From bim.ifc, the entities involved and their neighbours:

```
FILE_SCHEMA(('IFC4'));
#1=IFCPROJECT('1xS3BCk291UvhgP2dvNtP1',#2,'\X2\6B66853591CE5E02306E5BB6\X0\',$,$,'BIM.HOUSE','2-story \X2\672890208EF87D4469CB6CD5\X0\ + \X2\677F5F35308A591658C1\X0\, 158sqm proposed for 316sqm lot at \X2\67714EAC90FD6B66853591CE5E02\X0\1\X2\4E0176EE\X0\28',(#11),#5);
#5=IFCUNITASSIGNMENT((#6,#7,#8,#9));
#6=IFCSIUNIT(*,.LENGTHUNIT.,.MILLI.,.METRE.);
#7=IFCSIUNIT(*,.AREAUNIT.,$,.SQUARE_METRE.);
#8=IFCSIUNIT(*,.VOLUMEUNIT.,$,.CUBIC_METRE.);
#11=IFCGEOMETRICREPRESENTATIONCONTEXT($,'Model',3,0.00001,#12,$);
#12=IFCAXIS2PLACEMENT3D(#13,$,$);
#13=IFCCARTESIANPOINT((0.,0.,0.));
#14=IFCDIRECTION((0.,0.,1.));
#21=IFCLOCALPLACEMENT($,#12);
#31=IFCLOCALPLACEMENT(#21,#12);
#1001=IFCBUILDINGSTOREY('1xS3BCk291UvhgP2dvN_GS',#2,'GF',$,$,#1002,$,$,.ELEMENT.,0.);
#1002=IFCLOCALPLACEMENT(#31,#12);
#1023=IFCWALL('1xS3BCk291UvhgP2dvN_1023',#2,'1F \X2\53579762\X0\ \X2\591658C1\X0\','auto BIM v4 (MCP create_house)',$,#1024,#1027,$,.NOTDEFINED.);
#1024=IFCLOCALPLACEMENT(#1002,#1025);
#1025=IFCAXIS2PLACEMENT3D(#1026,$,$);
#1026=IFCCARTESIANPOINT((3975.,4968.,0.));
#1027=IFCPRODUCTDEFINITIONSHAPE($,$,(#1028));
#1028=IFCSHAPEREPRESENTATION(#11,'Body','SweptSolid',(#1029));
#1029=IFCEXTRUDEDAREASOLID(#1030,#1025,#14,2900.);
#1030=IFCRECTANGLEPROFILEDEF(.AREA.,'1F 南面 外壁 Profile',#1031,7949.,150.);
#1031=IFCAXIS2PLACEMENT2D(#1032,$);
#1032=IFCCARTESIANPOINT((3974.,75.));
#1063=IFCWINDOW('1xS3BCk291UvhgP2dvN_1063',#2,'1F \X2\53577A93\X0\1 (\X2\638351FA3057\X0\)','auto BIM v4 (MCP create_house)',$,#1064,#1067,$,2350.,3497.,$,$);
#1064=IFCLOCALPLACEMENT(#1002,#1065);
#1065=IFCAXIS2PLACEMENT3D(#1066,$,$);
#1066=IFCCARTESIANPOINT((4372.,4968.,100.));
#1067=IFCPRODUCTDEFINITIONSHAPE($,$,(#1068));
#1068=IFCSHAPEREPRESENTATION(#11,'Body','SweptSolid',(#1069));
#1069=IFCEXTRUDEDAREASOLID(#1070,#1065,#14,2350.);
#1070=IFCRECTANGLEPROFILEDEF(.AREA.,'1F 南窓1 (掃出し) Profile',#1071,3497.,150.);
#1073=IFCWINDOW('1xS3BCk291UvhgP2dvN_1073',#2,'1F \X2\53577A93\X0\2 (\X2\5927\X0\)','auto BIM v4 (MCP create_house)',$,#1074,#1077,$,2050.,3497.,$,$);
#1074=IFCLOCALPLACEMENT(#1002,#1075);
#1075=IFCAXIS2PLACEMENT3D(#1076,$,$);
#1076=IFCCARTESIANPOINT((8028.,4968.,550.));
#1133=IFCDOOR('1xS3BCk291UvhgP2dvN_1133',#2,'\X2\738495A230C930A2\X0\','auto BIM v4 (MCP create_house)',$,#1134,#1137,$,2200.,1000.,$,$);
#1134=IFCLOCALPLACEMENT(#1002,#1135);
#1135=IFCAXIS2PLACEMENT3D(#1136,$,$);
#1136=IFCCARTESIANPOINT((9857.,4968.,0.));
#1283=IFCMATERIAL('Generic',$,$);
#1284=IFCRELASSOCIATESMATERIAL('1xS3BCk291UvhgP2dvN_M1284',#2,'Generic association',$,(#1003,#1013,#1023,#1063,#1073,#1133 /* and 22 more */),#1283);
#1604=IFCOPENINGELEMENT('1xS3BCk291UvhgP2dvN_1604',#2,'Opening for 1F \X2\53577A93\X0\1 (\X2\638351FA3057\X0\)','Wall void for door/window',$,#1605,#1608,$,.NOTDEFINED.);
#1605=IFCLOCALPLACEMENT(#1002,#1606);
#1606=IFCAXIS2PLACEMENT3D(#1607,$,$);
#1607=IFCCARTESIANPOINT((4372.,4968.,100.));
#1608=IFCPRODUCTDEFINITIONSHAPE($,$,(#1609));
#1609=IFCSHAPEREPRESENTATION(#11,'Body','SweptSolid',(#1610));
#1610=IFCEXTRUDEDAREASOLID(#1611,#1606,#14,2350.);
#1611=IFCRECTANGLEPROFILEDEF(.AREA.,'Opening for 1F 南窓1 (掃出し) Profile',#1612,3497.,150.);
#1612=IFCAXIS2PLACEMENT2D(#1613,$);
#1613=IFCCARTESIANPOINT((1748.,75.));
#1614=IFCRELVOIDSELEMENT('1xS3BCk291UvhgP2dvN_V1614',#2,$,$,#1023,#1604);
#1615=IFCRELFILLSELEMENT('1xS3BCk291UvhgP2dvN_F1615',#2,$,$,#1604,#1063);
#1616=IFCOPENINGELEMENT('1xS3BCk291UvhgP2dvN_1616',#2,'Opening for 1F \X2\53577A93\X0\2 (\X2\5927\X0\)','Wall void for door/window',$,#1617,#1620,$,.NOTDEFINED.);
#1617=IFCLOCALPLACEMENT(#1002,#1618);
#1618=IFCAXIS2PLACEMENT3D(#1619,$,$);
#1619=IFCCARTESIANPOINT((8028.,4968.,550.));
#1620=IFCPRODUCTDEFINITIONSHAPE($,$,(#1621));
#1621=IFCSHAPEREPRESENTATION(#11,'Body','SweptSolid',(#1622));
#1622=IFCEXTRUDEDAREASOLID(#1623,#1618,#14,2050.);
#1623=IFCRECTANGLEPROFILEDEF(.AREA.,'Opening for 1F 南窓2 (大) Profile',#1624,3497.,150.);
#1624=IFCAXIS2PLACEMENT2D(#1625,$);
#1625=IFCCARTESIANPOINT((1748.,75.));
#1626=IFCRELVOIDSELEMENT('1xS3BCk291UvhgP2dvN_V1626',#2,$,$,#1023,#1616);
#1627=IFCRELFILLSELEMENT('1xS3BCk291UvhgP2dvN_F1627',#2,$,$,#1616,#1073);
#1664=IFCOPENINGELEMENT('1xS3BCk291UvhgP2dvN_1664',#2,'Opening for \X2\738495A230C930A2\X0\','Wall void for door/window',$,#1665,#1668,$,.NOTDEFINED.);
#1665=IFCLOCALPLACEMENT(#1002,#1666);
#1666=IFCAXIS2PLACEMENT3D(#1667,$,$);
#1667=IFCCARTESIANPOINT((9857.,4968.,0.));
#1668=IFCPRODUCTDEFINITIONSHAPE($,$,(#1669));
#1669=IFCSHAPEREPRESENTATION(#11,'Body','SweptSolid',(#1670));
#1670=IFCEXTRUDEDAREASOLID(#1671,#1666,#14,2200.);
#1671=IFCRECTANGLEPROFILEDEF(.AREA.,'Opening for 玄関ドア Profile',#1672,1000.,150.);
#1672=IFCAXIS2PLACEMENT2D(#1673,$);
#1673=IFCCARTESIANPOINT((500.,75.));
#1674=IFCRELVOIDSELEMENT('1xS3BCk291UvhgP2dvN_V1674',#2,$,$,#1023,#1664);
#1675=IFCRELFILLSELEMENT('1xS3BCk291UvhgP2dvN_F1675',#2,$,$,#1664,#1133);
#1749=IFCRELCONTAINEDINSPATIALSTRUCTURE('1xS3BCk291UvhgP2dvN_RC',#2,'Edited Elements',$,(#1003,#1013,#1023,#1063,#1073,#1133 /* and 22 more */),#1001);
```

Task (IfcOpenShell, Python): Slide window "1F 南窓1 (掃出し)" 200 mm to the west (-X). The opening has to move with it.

```python
import ifcopenshell
import ifcopenshell.api.geometry
import ifcopenshell.util.placement
import ifcopenshell.util.unit

model = ifcopenshell.open("bim.ifc")
unit_scale = ifcopenshell.util.unit.calculate_unit_scale(model)

window = model.by_guid("1xS3BCk291UvhgP2dvN_1063")
opening = window.FillsVoids[0].RelatingOpeningElement
wall = opening.VoidsElements[0].RelatingBuildingElement

wall_matrix = ifcopenshell.util.placement.get_local_placement(wall.ObjectPlacement)
shift = wall_matrix[:3, 0] * -0.2 / unit_scale
before = ifcopenshell.util.placement.get_local_placement(window.ObjectPlacement)[:3, 3].copy()

# The window is not placed relative to its opening, so move both.
for product in (opening, window):
    matrix = ifcopenshell.util.placement.get_local_placement(product.ObjectPlacement)
    matrix[:3, 3] += shift
    ifcopenshell.api.geometry.edit_object_placement(model, product=product, matrix=matrix, is_si=False)

after = ifcopenshell.util.placement.get_local_placement(window.ObjectPlacement)[:3, 3]
print("window moved by", (after - before).round(3) + 0.0)

model.write("bim_edited.ifc")
```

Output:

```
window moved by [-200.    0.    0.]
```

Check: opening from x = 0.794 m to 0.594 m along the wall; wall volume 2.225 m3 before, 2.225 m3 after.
